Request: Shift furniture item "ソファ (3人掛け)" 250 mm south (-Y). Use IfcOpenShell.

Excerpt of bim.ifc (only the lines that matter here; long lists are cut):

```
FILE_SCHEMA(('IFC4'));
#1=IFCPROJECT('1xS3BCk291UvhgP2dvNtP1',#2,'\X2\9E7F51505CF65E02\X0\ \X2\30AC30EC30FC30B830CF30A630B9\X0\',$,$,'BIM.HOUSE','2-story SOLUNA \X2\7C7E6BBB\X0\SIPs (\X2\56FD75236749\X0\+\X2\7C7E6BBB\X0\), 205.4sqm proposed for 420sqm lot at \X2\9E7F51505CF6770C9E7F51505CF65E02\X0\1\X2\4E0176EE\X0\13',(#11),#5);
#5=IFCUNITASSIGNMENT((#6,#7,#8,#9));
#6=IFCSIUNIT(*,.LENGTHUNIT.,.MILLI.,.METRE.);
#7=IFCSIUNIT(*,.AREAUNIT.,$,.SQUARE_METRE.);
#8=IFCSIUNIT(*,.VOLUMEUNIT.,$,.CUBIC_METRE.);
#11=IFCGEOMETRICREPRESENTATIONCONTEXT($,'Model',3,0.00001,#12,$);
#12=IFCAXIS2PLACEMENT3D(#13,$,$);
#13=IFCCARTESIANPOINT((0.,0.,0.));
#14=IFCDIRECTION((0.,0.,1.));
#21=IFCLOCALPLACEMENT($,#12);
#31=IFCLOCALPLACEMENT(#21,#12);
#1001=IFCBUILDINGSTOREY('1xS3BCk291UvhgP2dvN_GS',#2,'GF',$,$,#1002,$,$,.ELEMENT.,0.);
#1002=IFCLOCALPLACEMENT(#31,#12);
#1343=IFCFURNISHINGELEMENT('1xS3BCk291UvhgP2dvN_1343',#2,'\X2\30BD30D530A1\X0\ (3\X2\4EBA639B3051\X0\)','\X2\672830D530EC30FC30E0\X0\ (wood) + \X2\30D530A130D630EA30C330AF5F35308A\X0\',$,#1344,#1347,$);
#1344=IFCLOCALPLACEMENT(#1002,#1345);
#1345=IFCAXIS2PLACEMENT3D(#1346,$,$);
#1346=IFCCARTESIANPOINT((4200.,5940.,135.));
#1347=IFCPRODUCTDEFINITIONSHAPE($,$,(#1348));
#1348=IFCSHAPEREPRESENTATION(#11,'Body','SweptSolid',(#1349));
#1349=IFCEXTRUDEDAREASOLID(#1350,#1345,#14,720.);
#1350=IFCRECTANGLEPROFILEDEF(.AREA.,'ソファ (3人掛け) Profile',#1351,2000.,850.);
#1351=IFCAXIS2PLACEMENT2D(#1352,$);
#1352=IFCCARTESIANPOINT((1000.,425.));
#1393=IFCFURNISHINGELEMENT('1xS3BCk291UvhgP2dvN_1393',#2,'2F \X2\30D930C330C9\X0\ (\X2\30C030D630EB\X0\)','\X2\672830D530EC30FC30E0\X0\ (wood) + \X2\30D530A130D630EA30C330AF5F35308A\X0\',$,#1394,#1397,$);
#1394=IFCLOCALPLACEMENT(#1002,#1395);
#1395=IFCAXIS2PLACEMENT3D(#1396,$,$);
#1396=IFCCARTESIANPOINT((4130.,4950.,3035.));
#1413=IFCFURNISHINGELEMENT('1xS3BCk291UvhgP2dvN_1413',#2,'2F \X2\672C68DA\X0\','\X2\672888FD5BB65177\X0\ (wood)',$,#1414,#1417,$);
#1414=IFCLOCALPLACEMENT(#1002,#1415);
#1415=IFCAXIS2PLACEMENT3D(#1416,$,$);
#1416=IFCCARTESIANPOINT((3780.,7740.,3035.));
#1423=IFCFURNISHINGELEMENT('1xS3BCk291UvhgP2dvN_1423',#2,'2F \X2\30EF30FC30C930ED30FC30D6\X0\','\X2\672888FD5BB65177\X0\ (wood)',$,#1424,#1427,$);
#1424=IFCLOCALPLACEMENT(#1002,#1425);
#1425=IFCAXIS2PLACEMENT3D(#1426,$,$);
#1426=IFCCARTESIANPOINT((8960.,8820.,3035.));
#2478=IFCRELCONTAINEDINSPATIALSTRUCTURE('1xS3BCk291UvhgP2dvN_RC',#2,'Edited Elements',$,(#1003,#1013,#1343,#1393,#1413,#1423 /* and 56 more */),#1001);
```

```python
import ifcopenshell
import ifcopenshell.api.geometry
import ifcopenshell.util.placement
import ifcopenshell.util.unit

model = ifcopenshell.open("bim.ifc")
unit_scale = ifcopenshell.util.unit.calculate_unit_scale(model)

item = model.by_guid("1xS3BCk291UvhgP2dvN_1343")
matrix = ifcopenshell.util.placement.get_local_placement(item.ObjectPlacement)
matrix[1, 3] -= 0.25 / unit_scale
ifcopenshell.api.geometry.edit_object_placement(model, product=item, matrix=matrix, is_si=False)

print(ifcopenshell.util.placement.get_local_placement(item.ObjectPlacement).round(3) + 0.0)

model.write("bim_rev.ifc")
```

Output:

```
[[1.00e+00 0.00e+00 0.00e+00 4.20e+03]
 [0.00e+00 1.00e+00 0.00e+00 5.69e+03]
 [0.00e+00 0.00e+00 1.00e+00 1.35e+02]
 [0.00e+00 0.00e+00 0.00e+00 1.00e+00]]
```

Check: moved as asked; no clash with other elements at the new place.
